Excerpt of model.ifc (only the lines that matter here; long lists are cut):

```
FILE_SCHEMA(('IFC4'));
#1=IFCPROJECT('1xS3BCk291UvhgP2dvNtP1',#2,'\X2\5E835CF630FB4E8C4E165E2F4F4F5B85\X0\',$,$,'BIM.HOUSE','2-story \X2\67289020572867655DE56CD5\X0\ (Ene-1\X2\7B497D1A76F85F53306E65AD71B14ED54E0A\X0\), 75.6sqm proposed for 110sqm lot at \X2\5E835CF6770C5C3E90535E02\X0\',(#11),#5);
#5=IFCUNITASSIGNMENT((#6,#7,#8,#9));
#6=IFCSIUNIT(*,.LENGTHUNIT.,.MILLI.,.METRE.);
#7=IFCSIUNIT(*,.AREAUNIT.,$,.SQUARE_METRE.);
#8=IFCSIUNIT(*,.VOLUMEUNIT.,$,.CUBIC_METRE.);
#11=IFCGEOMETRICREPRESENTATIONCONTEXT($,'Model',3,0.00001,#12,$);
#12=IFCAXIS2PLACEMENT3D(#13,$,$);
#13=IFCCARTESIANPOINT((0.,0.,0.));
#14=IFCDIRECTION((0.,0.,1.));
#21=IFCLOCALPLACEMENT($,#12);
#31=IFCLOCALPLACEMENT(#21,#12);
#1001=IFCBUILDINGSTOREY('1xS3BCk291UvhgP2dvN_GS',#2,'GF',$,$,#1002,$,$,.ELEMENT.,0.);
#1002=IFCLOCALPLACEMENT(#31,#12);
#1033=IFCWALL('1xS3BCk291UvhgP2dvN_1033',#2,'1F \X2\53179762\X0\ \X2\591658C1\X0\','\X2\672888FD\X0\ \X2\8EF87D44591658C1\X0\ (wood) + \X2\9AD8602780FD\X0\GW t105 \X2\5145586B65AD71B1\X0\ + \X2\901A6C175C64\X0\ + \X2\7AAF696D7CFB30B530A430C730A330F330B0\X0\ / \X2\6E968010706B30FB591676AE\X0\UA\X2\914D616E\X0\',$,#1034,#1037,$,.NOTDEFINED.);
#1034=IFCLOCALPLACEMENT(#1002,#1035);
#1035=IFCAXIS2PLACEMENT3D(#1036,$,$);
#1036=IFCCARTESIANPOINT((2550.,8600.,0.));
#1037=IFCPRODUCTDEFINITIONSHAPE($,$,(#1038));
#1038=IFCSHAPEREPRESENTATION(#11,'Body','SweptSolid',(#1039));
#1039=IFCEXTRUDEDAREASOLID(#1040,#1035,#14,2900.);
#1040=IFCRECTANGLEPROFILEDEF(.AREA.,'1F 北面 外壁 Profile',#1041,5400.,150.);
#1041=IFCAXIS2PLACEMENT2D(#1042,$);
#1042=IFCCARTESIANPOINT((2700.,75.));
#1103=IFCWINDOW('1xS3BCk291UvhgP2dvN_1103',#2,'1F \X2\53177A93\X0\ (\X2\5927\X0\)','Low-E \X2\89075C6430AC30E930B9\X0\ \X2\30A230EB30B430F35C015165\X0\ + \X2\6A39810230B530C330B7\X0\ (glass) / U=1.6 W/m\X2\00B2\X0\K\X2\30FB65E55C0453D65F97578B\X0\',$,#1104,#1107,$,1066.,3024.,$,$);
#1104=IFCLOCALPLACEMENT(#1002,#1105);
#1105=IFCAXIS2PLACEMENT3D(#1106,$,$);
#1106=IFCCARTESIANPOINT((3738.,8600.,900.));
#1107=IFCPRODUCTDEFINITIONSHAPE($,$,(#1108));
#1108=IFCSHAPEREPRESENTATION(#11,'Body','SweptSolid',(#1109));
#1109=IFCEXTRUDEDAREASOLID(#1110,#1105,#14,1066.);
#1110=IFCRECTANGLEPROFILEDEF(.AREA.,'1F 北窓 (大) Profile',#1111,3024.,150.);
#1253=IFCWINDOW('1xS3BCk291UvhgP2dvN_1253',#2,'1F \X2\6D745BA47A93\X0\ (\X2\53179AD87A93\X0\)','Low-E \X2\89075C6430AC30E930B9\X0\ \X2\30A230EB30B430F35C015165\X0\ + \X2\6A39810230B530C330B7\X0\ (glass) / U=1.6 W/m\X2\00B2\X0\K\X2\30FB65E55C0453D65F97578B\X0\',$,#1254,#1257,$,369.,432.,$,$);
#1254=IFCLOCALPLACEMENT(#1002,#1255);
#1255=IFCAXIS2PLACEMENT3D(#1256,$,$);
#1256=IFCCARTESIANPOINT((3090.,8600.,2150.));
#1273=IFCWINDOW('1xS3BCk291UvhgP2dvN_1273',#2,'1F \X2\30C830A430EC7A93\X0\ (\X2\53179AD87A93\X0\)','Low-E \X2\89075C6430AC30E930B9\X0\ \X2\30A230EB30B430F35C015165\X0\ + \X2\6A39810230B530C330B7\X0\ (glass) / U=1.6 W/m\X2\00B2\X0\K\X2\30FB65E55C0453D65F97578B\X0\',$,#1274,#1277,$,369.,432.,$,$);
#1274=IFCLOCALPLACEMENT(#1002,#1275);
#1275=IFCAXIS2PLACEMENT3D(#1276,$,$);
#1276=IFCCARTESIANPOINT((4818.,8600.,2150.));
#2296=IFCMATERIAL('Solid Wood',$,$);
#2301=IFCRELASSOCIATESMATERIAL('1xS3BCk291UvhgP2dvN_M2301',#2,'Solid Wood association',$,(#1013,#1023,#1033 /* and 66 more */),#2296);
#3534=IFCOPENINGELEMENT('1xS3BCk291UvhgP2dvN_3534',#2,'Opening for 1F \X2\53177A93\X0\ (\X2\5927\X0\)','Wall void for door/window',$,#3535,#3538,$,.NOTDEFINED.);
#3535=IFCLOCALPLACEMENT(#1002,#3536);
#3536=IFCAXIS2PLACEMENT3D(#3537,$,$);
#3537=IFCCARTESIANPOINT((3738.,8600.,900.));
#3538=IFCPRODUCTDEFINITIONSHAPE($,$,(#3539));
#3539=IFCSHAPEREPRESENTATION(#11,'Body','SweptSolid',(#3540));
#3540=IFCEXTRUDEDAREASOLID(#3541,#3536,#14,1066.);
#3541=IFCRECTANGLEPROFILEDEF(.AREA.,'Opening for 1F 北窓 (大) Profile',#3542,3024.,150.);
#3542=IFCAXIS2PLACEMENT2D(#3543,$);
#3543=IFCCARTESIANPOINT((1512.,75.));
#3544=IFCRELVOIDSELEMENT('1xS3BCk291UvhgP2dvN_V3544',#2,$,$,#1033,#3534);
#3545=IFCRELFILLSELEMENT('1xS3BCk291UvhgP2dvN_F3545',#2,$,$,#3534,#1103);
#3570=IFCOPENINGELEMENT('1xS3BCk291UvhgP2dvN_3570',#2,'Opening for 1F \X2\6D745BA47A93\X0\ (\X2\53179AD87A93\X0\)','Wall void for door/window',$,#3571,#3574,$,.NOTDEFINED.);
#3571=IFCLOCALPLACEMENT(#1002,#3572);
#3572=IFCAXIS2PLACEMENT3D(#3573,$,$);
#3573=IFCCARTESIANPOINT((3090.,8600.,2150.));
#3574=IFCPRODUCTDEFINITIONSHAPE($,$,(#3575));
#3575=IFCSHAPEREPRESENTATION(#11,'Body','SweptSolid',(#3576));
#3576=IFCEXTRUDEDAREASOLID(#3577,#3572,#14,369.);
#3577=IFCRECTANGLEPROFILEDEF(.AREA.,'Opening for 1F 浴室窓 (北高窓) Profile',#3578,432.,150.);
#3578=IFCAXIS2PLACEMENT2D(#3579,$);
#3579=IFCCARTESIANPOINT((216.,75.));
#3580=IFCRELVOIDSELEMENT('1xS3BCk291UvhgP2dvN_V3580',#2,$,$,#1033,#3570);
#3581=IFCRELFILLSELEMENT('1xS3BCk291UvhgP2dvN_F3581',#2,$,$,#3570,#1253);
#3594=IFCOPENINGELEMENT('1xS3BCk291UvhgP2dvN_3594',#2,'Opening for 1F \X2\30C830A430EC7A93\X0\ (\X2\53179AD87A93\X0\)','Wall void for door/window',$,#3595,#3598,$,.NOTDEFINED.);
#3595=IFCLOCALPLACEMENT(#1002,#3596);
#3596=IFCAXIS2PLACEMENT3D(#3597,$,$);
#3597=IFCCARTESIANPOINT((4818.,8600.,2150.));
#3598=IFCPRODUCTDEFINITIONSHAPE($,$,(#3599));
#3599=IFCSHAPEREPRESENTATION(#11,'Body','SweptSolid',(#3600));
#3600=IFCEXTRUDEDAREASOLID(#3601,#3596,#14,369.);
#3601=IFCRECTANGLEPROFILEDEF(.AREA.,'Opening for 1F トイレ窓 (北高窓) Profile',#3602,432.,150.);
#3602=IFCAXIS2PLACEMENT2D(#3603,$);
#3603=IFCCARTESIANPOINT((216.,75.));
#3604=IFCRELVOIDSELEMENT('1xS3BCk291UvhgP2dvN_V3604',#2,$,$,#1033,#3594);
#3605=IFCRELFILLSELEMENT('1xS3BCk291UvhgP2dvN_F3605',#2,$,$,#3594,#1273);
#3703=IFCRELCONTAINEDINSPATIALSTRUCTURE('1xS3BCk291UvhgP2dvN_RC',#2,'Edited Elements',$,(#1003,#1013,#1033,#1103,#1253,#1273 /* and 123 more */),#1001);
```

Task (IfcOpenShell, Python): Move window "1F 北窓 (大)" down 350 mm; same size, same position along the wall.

```python
import numpy as np
import ifcopenshell
import ifcopenshell.api.geometry
import ifcopenshell.util.placement
import ifcopenshell.util.unit

model = ifcopenshell.open("model.ifc")
unit_scale = ifcopenshell.util.unit.calculate_unit_scale(model)

window = model.by_guid("1xS3BCk291UvhgP2dvN_1103")
opening = window.FillsVoids[0].RelatingOpeningElement
dz = -0.35 / unit_scale

shift = np.array([0.0, 0.0, dz])
# The window is not placed relative to its opening, so move both.
for product in (opening, window):
    matrix = ifcopenshell.util.placement.get_local_placement(product.ObjectPlacement)
    matrix[:3, 3] += shift
    ifcopenshell.api.geometry.edit_object_placement(model, product=product, matrix=matrix, is_si=False)

print(f"moved by {dz * unit_scale:+.3f} m")

model.write("model_rev.ifc")
```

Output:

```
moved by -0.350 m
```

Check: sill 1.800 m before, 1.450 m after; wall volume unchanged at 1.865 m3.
